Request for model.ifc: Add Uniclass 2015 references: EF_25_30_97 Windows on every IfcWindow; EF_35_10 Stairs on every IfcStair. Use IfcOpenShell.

First a look at what the model holds.

```python
import ifcopenshell

model = ifcopenshell.open("model.ifc")
print(model.schema)
print("classifications:", [c.Name for c in model.by_type("IfcClassification")])
for ifc_class in ("IfcDoor", "IfcRoof", "IfcStair", "IfcWall", "IfcWindow"):
    print(ifc_class, len(model.by_type(ifc_class)))
```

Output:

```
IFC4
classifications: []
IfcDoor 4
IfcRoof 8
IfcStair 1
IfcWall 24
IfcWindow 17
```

```python
import ifcopenshell
import ifcopenshell.api.classification

model = ifcopenshell.open("model.ifc")

system = ifcopenshell.api.classification.add_classification(model, classification="Uniclass 2015")

codes = {
    "IfcWindow": ("EF_25_30_97", "Windows"),
    "IfcStair": ("EF_35_10", "Stairs"),
}
for ifc_class, (code, name) in codes.items():
    products = model.by_type(ifc_class)
    ifcopenshell.api.classification.add_reference(
        model, products=products, classification=system, identification=code, name=name
    )
    print(code, len(products))

model.write("model_updated.ifc")
```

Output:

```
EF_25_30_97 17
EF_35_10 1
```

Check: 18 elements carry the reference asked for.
